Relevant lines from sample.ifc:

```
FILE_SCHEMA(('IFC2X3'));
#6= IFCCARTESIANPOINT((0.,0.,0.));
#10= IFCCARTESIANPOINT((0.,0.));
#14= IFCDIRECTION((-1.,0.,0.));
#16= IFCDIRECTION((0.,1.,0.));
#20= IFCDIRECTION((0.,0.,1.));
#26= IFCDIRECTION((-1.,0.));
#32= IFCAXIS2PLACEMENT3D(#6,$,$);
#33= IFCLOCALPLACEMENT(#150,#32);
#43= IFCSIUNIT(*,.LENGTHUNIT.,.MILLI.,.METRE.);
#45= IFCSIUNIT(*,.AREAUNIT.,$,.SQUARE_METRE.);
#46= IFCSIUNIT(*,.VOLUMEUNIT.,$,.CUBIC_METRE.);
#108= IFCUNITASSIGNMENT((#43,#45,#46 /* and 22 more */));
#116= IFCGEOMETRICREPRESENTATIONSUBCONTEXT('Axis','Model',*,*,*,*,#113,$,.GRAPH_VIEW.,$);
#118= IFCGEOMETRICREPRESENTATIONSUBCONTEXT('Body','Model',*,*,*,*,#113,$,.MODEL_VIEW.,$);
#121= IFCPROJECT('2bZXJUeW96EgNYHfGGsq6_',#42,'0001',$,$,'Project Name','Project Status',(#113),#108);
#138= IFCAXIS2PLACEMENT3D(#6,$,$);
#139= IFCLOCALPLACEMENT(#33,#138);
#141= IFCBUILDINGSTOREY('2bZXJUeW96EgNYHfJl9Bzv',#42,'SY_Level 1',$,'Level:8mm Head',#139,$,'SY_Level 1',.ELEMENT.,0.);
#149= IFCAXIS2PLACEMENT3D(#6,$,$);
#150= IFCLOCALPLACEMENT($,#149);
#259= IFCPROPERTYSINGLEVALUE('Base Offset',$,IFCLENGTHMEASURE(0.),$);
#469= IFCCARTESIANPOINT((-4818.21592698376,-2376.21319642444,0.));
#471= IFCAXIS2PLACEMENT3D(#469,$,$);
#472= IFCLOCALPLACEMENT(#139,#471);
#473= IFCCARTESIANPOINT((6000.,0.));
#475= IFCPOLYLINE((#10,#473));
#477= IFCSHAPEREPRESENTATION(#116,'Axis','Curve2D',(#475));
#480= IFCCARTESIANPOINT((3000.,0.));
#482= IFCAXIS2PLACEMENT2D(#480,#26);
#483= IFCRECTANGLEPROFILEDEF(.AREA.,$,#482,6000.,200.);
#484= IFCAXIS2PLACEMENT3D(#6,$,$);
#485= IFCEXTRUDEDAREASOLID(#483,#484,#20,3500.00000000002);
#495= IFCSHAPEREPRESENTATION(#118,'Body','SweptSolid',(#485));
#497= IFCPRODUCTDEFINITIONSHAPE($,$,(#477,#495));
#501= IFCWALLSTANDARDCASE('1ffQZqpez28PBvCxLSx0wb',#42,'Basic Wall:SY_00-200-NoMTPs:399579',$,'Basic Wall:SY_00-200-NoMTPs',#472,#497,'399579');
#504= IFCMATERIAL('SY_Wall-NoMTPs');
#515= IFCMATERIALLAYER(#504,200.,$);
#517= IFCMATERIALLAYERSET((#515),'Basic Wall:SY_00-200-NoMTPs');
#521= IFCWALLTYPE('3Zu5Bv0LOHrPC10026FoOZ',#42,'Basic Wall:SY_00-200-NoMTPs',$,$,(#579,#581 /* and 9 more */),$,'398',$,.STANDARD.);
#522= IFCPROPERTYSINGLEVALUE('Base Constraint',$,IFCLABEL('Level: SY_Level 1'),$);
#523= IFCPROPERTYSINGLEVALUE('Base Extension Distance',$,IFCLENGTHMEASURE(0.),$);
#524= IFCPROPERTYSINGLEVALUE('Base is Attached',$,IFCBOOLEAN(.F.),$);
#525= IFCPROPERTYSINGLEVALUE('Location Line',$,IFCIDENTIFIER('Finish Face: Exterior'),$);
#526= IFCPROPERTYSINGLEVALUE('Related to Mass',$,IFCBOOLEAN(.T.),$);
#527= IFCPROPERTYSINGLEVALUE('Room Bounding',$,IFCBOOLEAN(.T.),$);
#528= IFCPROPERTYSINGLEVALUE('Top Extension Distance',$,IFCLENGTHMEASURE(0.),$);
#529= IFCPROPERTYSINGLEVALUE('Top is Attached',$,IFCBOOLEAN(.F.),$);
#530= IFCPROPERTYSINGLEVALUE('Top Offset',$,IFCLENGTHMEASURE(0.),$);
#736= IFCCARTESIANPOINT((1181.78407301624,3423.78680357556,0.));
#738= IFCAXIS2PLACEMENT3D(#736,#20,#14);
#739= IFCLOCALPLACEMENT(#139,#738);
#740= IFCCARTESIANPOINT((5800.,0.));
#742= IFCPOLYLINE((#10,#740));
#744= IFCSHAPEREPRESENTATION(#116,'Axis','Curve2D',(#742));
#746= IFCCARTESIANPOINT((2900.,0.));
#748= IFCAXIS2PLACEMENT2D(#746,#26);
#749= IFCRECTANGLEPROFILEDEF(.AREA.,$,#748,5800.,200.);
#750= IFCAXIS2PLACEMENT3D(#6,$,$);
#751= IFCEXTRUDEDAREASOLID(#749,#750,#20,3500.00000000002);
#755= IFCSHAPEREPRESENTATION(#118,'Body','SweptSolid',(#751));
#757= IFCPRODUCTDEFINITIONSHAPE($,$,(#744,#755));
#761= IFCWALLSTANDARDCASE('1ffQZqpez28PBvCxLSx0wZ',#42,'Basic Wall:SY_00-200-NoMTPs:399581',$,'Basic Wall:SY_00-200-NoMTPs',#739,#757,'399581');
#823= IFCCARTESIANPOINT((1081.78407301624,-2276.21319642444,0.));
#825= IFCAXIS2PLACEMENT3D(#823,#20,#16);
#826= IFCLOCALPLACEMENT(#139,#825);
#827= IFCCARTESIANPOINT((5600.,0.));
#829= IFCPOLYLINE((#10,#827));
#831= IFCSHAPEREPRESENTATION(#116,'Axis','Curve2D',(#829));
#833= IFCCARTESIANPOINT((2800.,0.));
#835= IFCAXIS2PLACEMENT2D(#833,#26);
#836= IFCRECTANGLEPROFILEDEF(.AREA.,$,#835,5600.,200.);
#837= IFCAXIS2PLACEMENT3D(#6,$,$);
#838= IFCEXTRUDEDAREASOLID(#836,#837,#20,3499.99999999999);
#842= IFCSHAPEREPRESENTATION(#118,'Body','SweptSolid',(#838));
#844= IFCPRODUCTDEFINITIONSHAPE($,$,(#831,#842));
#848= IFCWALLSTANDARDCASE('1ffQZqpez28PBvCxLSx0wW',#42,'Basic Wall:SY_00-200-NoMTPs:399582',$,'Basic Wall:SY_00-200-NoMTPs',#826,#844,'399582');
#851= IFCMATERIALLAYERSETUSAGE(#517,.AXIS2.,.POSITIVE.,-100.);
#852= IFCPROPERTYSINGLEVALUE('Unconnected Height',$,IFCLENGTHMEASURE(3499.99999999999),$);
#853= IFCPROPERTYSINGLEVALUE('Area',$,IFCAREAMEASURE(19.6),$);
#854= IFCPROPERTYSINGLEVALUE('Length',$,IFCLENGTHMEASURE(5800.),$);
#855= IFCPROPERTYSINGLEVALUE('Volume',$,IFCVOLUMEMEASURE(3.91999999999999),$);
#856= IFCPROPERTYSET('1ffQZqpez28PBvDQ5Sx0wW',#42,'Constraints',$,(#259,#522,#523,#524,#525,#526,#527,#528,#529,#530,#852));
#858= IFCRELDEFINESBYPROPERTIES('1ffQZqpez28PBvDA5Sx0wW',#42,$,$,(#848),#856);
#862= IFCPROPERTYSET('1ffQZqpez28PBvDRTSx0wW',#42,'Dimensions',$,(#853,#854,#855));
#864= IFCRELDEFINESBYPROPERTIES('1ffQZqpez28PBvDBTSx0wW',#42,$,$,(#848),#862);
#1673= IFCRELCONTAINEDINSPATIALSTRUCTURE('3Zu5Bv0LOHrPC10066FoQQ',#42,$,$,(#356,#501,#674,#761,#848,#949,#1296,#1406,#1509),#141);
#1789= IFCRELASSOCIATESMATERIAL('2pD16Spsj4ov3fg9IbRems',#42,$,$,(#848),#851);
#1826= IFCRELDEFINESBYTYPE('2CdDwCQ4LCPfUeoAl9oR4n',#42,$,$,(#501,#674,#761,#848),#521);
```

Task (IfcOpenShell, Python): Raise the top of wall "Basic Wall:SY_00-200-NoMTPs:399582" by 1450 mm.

```python
import ifcopenshell
import ifcopenshell.api.pset
import ifcopenshell.geom
import ifcopenshell.util.element
import ifcopenshell.util.representation
import ifcopenshell.util.shape
import ifcopenshell.util.unit

model = ifcopenshell.open("sample.ifc")
unit_scale = ifcopenshell.util.unit.calculate_unit_scale(model)
area_scale = ifcopenshell.util.unit.calculate_unit_scale(model, "AREAUNIT")
volume_scale = ifcopenshell.util.unit.calculate_unit_scale(model, "VOLUMEUNIT")
settings = ifcopenshell.geom.settings()


def volume(element):
    """Net volume in cubic metres, openings subtracted."""
    shape = ifcopenshell.geom.create_shape(settings, element)
    return ifcopenshell.util.shape.get_volume(shape.geometry)


wall = model.by_guid("1ffQZqpez28PBvCxLSx0wW")
before = volume(wall)

body = ifcopenshell.util.representation.get_representation(wall, "Model", "Body")
solid = body.Items[0]
old_height = solid.Depth
solid.Depth += 1.45 / unit_scale
after = volume(wall)
thickness = 0.2  # wall thickness in metres

# Update the stored height, areas and volumes.
pset = model.by_id(ifcopenshell.util.element.get_pset(wall, "Constraints", should_inherit=False)["id"])
ifcopenshell.api.pset.edit_pset(model, pset=pset, properties={
    "Unconnected Height": model.create_entity("IfcLengthMeasure", solid.Depth),
})
pset = model.by_id(ifcopenshell.util.element.get_pset(wall, "Dimensions", should_inherit=False)["id"])
ifcopenshell.api.pset.edit_pset(model, pset=pset, properties={
    "Area": model.create_entity("IfcAreaMeasure", after / thickness / area_scale),
    "Volume": model.create_entity("IfcVolumeMeasure", after / volume_scale),
})

print(f"height {old_height:g} -> {solid.Depth:g}, volume {before:.3f} -> {after:.3f} m3")

model.write("sample_edited.ifc")
```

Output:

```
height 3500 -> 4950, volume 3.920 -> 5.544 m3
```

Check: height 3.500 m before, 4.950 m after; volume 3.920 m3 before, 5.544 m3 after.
